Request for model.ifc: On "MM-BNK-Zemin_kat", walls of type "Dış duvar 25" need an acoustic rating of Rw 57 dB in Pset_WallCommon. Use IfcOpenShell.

First a look at what the model holds.

```python
import ifcopenshell
import ifcopenshell.util.element

model = ifcopenshell.open("model.ifc")
print(model.schema)
storey = next(s for s in model.by_type("IfcBuildingStorey") if s.Name == "MM-BNK-Zemin_kat")
walls = [e for e in ifcopenshell.util.element.get_decomposition(storey) if e.is_a("IfcWall")]
seen = {}
for e in walls:
    element_type = ifcopenshell.util.element.get_type(e)
    key = (element_type.Name if element_type != e and element_type else None, ifcopenshell.util.element.get_pset(e, "Pset_WallCommon", "AcousticRating"))
    seen[key] = seen.get(key, 0) + 1
for (name, value), count in sorted(seen.items(), key=str):
    print(count, "x", name, "|", value)
```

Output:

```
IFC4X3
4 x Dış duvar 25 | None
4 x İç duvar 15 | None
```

```python
import ifcopenshell
import ifcopenshell.api.pset
import ifcopenshell.util.element

model = ifcopenshell.open("model.ifc")

storey = next(s for s in model.by_type("IfcBuildingStorey") if s.Name == "MM-BNK-Zemin_kat")
walls = [e for e in ifcopenshell.util.element.get_decomposition(storey) if e.is_a("IfcWall")]

count = 0
for e in walls:
    element_type = ifcopenshell.util.element.get_type(e)
    if element_type in (None, e) or element_type.Name != "Dış duvar 25":
        continue
    # add_pset returns the element's existing set when there is one.
    pset = ifcopenshell.api.pset.add_pset(model, product=e, name="Pset_WallCommon")
    ifcopenshell.api.pset.edit_pset(model, pset=pset, properties={"AcousticRating": "Rw 57 dB"})
    count += 1

print(count, "walls updated")

model.write("model_v2.ifc")
```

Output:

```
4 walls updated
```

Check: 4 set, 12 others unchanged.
